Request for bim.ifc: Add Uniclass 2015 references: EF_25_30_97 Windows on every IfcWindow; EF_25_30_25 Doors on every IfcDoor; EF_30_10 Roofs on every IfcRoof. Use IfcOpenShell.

First a look at what the model holds.

```python
import ifcopenshell

model = ifcopenshell.open("bim.ifc")
print(model.schema)
print("classifications:", [c.Name for c in model.by_type("IfcClassification")])
for ifc_class in ("IfcDoor", "IfcRoof", "IfcStair", "IfcWall", "IfcWindow"):
    print(ifc_class, len(model.by_type(ifc_class)))
```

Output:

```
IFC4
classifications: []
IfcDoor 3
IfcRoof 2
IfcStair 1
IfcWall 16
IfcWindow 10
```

```python
import ifcopenshell
import ifcopenshell.api.classification

model = ifcopenshell.open("bim.ifc")

system = ifcopenshell.api.classification.add_classification(model, classification="Uniclass 2015")

codes = {
    "IfcWindow": ("EF_25_30_97", "Windows"),
    "IfcDoor": ("EF_25_30_25", "Doors"),
    "IfcRoof": ("EF_30_10", "Roofs"),
}
for ifc_class, (code, name) in codes.items():
    products = model.by_type(ifc_class)
    ifcopenshell.api.classification.add_reference(
        model, products=products, classification=system, identification=code, name=name
    )
    print(code, len(products))

model.write("bim_v2.ifc")
```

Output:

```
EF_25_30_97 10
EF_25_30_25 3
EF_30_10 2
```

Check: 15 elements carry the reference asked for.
